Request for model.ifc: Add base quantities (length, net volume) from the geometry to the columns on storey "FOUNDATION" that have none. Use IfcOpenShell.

First a look at what the model holds.

```python
import ifcopenshell
import ifcopenshell.util.element
import ifcopenshell.util.unit

model = ifcopenshell.open("model.ifc")
print(model.schema)
for unit_type in ("LENGTHUNIT", "AREAUNIT", "VOLUMEUNIT"):
    print(unit_type, ifcopenshell.util.unit.calculate_unit_scale(model, unit_type))
storey = next(s for s in model.by_type("IfcBuildingStorey") if s.Name == "FOUNDATION")
columns = [e for e in ifcopenshell.util.element.get_decomposition(storey) if e.is_a("IfcColumn")]
for e in sorted(columns, key=lambda e: e.id()):
    print(e.id(), e.is_a(), e.Name, list(ifcopenshell.util.element.get_psets(e, qtos_only=True)), sep=" | ")
```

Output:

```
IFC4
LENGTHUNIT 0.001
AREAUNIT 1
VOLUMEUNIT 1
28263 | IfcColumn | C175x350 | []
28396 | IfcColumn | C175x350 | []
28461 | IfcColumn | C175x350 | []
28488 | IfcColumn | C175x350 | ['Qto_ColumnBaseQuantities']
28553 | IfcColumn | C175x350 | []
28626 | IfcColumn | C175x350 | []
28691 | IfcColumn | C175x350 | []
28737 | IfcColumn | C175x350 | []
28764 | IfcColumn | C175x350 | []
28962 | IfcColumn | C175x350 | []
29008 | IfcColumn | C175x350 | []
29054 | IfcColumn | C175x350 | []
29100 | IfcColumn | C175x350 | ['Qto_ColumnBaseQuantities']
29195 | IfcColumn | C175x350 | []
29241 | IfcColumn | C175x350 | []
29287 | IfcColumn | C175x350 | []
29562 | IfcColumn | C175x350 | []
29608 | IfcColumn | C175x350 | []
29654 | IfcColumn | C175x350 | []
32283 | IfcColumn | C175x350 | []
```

```python
import ifcopenshell
import ifcopenshell.api.pset
import ifcopenshell.geom
import ifcopenshell.util.element
import ifcopenshell.util.shape
import ifcopenshell.util.unit

model = ifcopenshell.open("model.ifc")
unit_scale = ifcopenshell.util.unit.calculate_unit_scale(model)
volume_scale = ifcopenshell.util.unit.calculate_unit_scale(model, "VOLUMEUNIT")
settings = ifcopenshell.geom.settings()

storey = next(s for s in model.by_type("IfcBuildingStorey") if s.Name == "FOUNDATION")
columns = [e for e in ifcopenshell.util.element.get_decomposition(storey) if e.is_a("IfcColumn")]

for e in sorted(columns, key=lambda e: e.id()):
    if ifcopenshell.util.element.get_psets(e, qtos_only=True, should_inherit=False):
        continue
    # Geometry comes back in metres, in the element's own axes.
    shape = ifcopenshell.geom.create_shape(settings, e)
    values = {
        "Length": ifcopenshell.util.shape.get_z(shape.geometry) / unit_scale,
        "NetVolume": ifcopenshell.util.shape.get_volume(shape.geometry) / volume_scale,
    }
    qto = ifcopenshell.api.pset.add_qto(model, product=e, name="Qto_ColumnBaseQuantities")
    ifcopenshell.api.pset.edit_qto(model, qto=qto, properties=values)
    print(e.id(), {k: round(v, 3) for k, v in values.items()})

model.write("model_v2.ifc")
```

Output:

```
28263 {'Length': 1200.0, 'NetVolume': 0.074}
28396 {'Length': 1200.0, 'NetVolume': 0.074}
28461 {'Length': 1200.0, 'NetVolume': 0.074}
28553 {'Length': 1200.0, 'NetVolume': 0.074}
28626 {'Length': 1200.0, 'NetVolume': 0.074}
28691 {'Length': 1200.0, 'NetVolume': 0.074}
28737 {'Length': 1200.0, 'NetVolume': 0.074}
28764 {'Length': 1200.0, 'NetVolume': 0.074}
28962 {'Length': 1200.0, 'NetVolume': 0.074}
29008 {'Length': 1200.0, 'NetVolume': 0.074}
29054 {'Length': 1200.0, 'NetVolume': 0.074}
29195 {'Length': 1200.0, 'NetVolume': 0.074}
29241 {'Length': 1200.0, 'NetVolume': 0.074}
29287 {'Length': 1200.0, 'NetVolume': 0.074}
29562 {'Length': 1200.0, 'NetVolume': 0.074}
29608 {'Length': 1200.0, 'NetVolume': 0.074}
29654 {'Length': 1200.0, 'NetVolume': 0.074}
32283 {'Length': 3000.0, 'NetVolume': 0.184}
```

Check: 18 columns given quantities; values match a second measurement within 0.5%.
